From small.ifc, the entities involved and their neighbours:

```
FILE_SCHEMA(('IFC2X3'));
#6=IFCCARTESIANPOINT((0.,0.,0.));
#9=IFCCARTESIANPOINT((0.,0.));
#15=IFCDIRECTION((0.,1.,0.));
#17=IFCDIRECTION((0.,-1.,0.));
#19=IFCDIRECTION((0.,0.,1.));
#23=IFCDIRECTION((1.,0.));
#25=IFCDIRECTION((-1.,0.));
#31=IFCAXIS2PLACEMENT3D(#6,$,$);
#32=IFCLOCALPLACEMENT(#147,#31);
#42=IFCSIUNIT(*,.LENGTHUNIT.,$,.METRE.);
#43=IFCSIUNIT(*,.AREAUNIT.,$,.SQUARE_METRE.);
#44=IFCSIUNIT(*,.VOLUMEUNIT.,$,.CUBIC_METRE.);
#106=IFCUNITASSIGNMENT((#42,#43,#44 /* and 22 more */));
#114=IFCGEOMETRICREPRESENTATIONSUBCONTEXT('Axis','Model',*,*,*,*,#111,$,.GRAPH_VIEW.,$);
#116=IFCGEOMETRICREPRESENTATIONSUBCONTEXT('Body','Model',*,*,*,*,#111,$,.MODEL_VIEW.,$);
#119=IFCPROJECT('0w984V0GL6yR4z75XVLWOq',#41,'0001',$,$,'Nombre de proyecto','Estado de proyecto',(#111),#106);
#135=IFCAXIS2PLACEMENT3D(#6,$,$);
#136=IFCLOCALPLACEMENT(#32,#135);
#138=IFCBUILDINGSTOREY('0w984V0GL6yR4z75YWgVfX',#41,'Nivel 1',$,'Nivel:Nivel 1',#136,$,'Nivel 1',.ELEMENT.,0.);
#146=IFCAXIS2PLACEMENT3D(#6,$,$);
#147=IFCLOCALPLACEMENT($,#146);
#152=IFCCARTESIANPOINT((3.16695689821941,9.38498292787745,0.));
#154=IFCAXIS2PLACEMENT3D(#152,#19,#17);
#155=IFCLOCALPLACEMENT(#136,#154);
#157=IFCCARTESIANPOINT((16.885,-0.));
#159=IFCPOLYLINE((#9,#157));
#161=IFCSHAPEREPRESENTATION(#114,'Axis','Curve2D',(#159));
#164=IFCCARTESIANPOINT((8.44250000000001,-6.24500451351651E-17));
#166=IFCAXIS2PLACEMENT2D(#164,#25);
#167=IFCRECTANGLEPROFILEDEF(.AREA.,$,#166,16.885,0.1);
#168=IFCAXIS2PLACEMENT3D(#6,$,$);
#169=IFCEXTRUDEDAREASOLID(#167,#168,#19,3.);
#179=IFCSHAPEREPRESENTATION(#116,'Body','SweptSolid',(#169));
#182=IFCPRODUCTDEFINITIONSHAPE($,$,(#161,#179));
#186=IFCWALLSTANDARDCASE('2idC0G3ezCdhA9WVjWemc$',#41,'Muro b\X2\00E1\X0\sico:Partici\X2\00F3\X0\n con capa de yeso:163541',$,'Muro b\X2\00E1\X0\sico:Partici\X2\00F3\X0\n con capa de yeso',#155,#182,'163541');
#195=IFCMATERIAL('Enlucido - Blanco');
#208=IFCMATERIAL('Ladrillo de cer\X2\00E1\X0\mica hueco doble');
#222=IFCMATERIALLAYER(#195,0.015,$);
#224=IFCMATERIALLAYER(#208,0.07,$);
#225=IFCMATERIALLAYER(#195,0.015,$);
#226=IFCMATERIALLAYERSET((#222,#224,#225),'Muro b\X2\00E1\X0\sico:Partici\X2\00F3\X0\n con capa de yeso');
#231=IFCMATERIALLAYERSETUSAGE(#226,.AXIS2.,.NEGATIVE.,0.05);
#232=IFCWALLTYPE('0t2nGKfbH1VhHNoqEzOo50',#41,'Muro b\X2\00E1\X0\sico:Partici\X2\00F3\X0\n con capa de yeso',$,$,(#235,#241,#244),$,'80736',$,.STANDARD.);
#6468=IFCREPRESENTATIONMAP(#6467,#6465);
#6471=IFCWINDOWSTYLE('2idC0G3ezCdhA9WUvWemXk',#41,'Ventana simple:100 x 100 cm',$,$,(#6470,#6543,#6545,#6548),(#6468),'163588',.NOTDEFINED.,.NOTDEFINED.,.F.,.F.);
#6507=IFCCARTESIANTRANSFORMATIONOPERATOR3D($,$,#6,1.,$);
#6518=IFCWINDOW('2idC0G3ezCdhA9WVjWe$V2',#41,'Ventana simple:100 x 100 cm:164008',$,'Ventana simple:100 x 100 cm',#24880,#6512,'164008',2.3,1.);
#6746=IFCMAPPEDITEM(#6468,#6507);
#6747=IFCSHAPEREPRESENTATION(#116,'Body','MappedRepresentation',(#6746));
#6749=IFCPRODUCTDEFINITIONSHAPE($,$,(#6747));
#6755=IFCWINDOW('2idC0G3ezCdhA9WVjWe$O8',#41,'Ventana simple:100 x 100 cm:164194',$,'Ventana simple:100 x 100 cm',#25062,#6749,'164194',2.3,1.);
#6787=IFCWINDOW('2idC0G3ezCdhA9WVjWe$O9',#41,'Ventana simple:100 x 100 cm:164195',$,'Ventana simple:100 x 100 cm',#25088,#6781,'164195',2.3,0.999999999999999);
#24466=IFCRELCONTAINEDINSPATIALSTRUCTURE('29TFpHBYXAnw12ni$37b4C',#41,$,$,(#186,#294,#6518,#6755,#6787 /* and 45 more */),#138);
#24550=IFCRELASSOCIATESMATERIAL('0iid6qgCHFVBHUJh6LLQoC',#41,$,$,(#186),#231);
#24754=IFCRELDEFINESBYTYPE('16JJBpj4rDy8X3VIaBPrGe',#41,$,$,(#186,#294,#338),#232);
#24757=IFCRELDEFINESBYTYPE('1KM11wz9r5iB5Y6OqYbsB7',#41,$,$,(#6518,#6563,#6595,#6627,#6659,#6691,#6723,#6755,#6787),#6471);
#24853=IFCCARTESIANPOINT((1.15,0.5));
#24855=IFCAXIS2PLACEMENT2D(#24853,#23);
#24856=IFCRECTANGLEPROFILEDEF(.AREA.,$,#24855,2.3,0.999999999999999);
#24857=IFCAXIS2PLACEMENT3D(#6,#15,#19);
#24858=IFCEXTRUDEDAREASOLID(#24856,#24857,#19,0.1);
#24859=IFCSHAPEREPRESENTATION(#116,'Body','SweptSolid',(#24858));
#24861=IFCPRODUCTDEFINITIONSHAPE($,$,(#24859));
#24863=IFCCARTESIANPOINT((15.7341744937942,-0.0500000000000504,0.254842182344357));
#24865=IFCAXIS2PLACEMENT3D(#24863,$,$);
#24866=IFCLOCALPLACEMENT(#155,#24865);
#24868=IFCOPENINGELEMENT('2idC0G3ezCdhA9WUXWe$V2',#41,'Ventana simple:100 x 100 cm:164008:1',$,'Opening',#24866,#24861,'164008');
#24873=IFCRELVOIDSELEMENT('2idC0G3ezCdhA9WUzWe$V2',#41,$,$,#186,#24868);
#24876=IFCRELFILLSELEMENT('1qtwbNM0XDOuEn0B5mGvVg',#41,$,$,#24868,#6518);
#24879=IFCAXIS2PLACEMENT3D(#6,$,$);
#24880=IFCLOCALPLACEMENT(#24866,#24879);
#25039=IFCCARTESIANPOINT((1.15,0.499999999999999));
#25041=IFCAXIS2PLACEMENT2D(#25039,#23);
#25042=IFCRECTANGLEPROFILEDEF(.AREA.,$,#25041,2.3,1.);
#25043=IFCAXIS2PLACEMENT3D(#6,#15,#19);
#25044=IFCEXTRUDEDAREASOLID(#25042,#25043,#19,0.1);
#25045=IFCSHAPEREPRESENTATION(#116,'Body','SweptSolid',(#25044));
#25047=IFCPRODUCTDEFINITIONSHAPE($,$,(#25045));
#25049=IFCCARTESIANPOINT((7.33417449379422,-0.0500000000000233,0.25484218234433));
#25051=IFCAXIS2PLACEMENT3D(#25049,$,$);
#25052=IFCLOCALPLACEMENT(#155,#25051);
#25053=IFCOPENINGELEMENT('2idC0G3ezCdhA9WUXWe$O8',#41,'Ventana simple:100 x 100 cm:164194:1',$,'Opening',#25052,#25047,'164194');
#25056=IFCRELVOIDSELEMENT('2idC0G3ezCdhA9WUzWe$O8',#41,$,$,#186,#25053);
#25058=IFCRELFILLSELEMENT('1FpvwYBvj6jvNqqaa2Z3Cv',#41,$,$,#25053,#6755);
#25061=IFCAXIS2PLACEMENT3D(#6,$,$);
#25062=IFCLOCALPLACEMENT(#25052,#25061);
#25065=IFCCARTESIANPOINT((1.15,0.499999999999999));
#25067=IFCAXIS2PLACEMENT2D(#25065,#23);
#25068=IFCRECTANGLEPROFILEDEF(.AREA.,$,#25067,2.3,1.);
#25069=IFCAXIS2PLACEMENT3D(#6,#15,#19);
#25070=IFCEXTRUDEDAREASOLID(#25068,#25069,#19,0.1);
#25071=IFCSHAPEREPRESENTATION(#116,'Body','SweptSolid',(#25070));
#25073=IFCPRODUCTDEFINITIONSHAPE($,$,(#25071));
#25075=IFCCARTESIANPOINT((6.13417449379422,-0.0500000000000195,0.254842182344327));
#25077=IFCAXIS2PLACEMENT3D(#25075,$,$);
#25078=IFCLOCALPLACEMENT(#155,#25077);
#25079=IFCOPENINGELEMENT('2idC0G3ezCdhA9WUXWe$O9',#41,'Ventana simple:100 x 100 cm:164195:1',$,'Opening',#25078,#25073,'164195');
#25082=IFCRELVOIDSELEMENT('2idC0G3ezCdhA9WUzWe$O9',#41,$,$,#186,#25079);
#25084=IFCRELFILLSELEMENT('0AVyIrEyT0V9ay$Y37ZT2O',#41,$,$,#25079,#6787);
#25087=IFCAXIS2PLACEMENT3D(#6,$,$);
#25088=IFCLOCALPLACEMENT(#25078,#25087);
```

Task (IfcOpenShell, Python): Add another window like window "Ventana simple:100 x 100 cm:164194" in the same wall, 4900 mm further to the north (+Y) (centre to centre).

```python
import ifcopenshell
import ifcopenshell.api.feature
import ifcopenshell.api.geometry
import ifcopenshell.api.root
import ifcopenshell.geom
import ifcopenshell.util.element
import ifcopenshell.util.placement
import ifcopenshell.util.shape
import ifcopenshell.util.unit

model = ifcopenshell.open("small.ifc")
unit_scale = ifcopenshell.util.unit.calculate_unit_scale(model)
settings = ifcopenshell.geom.settings()


def volume(element):
    """Net volume in cubic metres, openings subtracted."""
    shape = ifcopenshell.geom.create_shape(settings, element)
    return ifcopenshell.util.shape.get_volume(shape.geometry)


def reuse_history(source, copy):
    """copy_class also copies each property set's owner history, people and application; keep the originals."""
    for rel in copy.IsDefinedBy:
        if rel.is_a("IfcRelDefinesByProperties") and (history := rel.RelatingPropertyDefinition.OwnerHistory):
            rel.RelatingPropertyDefinition.OwnerHistory = source.OwnerHistory
            ifcopenshell.util.element.remove_deep2(model, history)


window = model.by_id(6755)
opening = window.FillsVoids[0].RelatingOpeningElement
wall = opening.VoidsElements[0].RelatingBuildingElement
before = volume(wall)
shift = ifcopenshell.util.placement.get_local_placement(wall.ObjectPlacement)[:3, 0] * -4.9 / unit_scale

# copy_class copies the void relationship, type, container and properties, but no geometry.
new_opening = ifcopenshell.api.root.copy_class(model, product=opening)
new_opening.Representation = ifcopenshell.util.element.copy_deep(
    model, opening.Representation, exclude=["IfcGeometricRepresentationContext", "IfcRepresentationMap"]
)
new_opening.Name = "Ventana simple:100 x 100 cm"
new_opening.Tag = None
new_window = ifcopenshell.api.root.copy_class(model, product=window)
new_window.Representation = ifcopenshell.util.element.copy_deep(
    model, window.Representation, exclude=["IfcGeometricRepresentationContext", "IfcRepresentationMap"]
)
new_window.Name = "Ventana simple:100 x 100 cm"
new_window.Tag = None
reuse_history(window, new_window)
fills = ifcopenshell.api.feature.add_filling(model, opening=new_opening, element=new_window)
fills.OwnerHistory = new_window.OwnerHistory  # required in IFC2X3

for old, new in ((opening, new_opening), (window, new_window)):
    matrix = ifcopenshell.util.placement.get_local_placement(old.ObjectPlacement)
    matrix[:3, 3] += shift
    ifcopenshell.api.geometry.edit_object_placement(model, product=new, matrix=matrix, is_si=False)

after = volume(wall)

print(f"wall volume {before:.3f} -> {after:.3f} m3")

model.write("small_edited.ifc")
```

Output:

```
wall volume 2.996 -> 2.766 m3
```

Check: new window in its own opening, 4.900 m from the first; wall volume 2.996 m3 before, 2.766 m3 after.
